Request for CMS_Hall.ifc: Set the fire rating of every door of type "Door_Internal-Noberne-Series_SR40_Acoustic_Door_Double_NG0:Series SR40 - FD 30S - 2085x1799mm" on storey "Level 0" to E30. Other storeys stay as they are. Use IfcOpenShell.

First a look at what the model holds.

```python
import ifcopenshell
import ifcopenshell.util.element

model = ifcopenshell.open("CMS_Hall.ifc")
print(model.schema)
storey = next(s for s in model.by_type("IfcBuildingStorey") if s.Name == "Level 0")
doors = [e for e in ifcopenshell.util.element.get_decomposition(storey) if e.is_a("IfcDoor")]
seen = {}
for e in doors:
    element_type = ifcopenshell.util.element.get_type(e)
    key = (element_type.Name if element_type != e and element_type else None, ifcopenshell.util.element.get_pset(e, "Pset_DoorCommon", "FireRating"))
    seen[key] = seen.get(key, 0) + 1
for (name, value), count in sorted(seen.items(), key=str):
    print(count, "x", name, "|", value)
```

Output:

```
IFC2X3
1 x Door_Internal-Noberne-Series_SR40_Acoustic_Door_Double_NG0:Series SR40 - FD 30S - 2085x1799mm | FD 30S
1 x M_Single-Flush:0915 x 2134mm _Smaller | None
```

```python
import ifcopenshell
import ifcopenshell.api.pset
import ifcopenshell.util.element

model = ifcopenshell.open("CMS_Hall.ifc")

storey = next(s for s in model.by_type("IfcBuildingStorey") if s.Name == "Level 0")
doors = [e for e in ifcopenshell.util.element.get_decomposition(storey) if e.is_a("IfcDoor")]

count = 0
for e in doors:
    element_type = ifcopenshell.util.element.get_type(e)
    if element_type in (None, e) or element_type.Name != "Door_Internal-Noberne-Series_SR40_Acoustic_Door_Double_NG0:Series SR40 - FD 30S - 2085x1799mm":
        continue
    # add_pset returns the element's existing set when there is one.
    pset = ifcopenshell.api.pset.add_pset(model, product=e, name="Pset_DoorCommon")
    ifcopenshell.api.pset.edit_pset(model, pset=pset, properties={"FireRating": "E30"})
    count += 1

print(count, "doors updated")

model.write("CMS_Hall_rev.ifc")
```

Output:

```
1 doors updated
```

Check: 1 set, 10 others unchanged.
